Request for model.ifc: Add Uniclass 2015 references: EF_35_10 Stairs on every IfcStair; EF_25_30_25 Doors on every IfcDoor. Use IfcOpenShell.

First a look at what the model holds.

```python
import ifcopenshell

model = ifcopenshell.open("model.ifc")
print(model.schema)
print("classifications:", [c.Name for c in model.by_type("IfcClassification")])
for ifc_class in ("IfcDoor", "IfcRoof", "IfcStair", "IfcWall", "IfcWindow"):
    print(ifc_class, len(model.by_type(ifc_class)))
```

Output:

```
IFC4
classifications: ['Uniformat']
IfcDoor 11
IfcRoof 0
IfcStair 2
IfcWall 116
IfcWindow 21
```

```python
import ifcopenshell
import ifcopenshell.api.classification

model = ifcopenshell.open("model.ifc")

system = ifcopenshell.api.classification.add_classification(model, classification="Uniclass 2015")

codes = {
    "IfcStair": ("EF_35_10", "Stairs"),
    "IfcDoor": ("EF_25_30_25", "Doors"),
}
for ifc_class, (code, name) in codes.items():
    products = model.by_type(ifc_class)
    ifcopenshell.api.classification.add_reference(
        model, products=products, classification=system, identification=code, name=name
    )
    print(code, len(products))

model.write("model_edited.ifc")
```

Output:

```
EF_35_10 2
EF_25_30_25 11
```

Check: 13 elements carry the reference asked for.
